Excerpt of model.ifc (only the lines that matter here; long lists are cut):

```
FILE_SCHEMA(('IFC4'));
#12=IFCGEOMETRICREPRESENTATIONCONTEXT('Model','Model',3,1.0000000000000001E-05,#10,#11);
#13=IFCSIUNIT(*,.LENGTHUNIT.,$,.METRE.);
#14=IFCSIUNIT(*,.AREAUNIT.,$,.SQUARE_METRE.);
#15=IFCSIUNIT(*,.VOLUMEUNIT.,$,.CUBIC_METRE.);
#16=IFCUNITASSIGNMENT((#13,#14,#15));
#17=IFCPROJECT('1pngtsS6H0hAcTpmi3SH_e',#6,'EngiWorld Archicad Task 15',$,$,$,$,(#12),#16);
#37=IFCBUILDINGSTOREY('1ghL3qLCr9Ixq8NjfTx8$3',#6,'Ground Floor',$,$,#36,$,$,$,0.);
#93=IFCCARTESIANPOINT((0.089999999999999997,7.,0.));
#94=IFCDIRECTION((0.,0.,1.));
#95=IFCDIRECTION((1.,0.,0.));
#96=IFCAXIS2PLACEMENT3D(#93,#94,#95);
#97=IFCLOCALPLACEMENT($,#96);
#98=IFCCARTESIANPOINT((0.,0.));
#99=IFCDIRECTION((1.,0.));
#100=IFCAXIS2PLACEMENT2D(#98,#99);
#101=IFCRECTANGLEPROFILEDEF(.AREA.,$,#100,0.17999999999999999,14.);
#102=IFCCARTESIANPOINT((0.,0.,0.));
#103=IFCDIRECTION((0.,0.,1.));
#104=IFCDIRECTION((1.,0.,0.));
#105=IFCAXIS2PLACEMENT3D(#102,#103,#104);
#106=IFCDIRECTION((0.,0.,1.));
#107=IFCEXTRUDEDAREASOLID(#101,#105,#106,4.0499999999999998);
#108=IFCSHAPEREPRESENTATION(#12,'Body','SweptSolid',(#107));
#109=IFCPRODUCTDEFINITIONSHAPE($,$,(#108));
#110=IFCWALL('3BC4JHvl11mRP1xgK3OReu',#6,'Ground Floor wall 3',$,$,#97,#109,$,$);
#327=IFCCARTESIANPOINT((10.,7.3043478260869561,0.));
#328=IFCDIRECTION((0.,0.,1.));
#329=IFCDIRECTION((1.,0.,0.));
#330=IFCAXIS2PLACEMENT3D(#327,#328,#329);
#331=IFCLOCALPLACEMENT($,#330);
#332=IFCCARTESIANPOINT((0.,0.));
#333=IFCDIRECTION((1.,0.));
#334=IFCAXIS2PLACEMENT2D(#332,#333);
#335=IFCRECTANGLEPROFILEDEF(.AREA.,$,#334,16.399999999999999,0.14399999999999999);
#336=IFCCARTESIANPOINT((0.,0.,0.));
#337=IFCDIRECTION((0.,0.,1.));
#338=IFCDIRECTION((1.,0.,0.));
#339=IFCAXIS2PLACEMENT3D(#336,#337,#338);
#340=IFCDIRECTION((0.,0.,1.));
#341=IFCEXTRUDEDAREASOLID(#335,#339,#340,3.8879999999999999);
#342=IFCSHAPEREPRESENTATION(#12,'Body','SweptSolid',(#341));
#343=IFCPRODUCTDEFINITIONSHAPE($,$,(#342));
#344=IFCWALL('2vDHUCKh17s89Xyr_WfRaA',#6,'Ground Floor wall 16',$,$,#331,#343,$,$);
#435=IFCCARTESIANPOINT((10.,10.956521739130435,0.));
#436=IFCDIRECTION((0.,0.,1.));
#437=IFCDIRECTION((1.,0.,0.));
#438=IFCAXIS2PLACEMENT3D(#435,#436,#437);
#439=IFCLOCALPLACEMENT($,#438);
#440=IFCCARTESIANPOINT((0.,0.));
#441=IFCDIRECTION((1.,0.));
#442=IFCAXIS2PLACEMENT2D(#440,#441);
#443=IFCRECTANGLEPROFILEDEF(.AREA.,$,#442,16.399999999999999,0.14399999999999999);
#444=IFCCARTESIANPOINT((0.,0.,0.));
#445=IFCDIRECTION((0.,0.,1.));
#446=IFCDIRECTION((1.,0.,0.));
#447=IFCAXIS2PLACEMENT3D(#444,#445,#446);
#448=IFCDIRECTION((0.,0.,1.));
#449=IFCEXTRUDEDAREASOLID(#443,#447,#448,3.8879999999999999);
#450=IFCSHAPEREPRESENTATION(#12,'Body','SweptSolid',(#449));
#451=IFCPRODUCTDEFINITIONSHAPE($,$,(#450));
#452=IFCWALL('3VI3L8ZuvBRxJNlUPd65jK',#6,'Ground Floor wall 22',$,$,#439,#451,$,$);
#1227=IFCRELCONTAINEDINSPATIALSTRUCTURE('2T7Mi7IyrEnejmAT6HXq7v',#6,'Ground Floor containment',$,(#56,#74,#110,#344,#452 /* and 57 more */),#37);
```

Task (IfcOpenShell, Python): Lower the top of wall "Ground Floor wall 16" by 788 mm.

```python
import ifcopenshell
import ifcopenshell.geom
import ifcopenshell.util.shape
import ifcopenshell.util.unit

model = ifcopenshell.open("model.ifc")
unit_scale = ifcopenshell.util.unit.calculate_unit_scale(model)
settings = ifcopenshell.geom.settings()


def volume(element):
    """Net volume in cubic metres, openings subtracted."""
    shape = ifcopenshell.geom.create_shape(settings, element)
    return ifcopenshell.util.shape.get_volume(shape.geometry)


wall = model.by_guid("2vDHUCKh17s89Xyr_WfRaA")
before = volume(wall)

body = next(r for r in wall.Representation.Representations if r.RepresentationIdentifier == "Body")
solid = body.Items[0]
old_height = solid.Depth
solid.Depth -= 0.788 / unit_scale
after = volume(wall)

print(f"height {old_height:g} -> {solid.Depth:g}, volume {before:.3f} -> {after:.3f} m3")

model.write("model_rev.ifc")
```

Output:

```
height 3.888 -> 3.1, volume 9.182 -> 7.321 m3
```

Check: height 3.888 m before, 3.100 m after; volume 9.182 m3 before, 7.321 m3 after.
